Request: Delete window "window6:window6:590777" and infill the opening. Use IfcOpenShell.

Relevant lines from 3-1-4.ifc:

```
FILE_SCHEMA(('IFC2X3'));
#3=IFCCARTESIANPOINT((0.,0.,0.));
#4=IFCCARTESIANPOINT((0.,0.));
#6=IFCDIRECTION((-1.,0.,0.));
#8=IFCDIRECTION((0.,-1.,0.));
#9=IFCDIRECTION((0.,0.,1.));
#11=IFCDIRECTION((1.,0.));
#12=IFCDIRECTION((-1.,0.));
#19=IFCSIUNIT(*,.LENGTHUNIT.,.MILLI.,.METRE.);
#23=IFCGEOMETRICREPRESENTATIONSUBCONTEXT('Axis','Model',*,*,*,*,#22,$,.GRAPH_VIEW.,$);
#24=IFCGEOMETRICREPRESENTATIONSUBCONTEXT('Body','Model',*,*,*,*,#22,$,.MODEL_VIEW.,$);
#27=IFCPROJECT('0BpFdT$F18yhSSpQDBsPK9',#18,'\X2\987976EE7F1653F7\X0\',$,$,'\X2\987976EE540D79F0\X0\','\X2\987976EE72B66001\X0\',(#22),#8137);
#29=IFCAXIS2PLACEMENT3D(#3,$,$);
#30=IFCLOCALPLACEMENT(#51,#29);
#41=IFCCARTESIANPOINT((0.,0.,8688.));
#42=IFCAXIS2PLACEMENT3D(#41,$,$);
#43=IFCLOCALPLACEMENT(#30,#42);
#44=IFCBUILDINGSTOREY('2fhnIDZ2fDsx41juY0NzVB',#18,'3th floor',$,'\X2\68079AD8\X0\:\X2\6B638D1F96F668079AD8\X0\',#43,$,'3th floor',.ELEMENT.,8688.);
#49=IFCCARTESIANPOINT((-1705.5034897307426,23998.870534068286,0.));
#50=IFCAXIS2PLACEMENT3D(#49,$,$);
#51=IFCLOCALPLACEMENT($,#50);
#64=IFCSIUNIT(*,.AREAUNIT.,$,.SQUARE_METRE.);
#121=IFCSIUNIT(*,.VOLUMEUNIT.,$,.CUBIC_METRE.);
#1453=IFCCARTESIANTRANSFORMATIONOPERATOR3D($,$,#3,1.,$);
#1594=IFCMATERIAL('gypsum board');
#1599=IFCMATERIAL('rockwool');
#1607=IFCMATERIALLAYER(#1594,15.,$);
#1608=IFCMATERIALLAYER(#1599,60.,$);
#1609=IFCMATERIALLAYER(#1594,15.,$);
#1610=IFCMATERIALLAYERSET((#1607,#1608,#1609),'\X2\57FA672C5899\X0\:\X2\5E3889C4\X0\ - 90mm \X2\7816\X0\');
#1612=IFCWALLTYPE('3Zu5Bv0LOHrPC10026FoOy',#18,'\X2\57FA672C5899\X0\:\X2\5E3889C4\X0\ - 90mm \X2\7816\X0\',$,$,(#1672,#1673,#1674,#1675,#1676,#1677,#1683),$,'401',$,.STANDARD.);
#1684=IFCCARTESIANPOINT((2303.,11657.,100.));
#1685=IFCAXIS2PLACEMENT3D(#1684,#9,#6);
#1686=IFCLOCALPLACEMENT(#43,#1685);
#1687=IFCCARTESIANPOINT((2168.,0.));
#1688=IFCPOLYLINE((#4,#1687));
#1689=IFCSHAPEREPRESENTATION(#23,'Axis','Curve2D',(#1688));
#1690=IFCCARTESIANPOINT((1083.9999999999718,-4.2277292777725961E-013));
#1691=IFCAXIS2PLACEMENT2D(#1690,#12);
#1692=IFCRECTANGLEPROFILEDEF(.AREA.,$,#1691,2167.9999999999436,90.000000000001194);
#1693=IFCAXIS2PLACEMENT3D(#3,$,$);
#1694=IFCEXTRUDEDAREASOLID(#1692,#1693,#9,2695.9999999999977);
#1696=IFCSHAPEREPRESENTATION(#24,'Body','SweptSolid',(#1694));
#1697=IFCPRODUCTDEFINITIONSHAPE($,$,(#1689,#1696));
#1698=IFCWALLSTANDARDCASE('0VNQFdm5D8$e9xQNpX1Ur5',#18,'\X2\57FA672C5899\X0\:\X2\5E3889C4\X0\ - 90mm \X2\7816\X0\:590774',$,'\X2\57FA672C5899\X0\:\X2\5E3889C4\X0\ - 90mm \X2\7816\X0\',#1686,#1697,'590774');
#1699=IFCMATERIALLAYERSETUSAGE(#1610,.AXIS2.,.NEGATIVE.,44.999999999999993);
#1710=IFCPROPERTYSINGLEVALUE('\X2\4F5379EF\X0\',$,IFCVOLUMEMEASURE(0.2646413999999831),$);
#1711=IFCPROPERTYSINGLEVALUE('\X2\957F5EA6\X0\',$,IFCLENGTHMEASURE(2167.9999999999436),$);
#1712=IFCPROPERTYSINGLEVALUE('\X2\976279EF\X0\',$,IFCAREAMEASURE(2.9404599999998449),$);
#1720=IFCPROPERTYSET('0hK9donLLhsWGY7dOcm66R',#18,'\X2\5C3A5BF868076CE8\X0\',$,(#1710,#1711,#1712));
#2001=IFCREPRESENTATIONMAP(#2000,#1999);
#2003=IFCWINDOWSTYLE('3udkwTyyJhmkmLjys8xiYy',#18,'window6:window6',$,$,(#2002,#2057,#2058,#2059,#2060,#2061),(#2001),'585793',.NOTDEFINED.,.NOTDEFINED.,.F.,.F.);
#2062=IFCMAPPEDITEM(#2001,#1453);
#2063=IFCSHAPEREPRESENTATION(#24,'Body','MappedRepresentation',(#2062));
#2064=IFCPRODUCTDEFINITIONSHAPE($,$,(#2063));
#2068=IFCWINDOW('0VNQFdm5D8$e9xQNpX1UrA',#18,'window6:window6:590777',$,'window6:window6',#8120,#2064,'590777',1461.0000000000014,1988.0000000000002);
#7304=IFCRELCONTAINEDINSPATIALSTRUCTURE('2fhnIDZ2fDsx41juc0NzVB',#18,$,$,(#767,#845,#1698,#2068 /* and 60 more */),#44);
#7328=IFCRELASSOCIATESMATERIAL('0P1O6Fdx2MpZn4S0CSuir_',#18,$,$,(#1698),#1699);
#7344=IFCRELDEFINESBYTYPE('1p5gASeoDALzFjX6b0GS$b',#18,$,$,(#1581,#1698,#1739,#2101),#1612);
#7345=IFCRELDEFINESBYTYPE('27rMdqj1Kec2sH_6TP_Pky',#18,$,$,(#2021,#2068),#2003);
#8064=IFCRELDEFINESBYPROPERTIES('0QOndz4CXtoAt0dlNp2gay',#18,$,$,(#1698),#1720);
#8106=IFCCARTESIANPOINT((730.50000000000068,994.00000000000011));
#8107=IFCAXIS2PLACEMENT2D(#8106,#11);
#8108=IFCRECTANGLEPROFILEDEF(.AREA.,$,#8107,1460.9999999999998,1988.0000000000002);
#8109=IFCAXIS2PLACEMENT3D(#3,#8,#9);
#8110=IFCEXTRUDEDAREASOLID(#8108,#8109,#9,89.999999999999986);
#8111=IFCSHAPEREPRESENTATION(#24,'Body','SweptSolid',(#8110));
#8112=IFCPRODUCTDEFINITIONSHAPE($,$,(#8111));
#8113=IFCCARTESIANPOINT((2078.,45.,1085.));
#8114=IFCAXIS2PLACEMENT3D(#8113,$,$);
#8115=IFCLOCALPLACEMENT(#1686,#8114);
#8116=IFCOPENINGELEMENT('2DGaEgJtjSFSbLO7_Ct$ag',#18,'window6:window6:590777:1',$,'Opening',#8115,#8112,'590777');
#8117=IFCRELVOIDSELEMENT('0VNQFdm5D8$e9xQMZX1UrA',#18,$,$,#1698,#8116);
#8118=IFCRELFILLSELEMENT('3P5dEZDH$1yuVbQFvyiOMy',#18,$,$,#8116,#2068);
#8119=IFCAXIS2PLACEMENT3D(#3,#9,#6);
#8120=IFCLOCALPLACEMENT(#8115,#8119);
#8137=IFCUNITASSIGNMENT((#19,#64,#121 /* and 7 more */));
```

```python
import ifcopenshell
import ifcopenshell.api.feature
import ifcopenshell.api.pset
import ifcopenshell.api.root
import ifcopenshell.geom
import ifcopenshell.util.element
import ifcopenshell.util.shape
import ifcopenshell.util.unit

model = ifcopenshell.open("3-1-4.ifc")
area_scale = ifcopenshell.util.unit.calculate_unit_scale(model, "AREAUNIT")
volume_scale = ifcopenshell.util.unit.calculate_unit_scale(model, "VOLUMEUNIT")
settings = ifcopenshell.geom.settings()


def volume(element):
    """Net volume in cubic metres, openings subtracted."""
    shape = ifcopenshell.geom.create_shape(settings, element)
    return ifcopenshell.util.shape.get_volume(shape.geometry)


window = model.by_id(2068)
opening = window.FillsVoids[0].RelatingOpeningElement
wall = opening.VoidsElements[0].RelatingBuildingElement
before = volume(wall)

ifcopenshell.api.root.remove_product(model, product=window)
ifcopenshell.api.feature.remove_feature(model, feature=opening)

after = volume(wall)
thickness = 0.09  # wall thickness in metres

# Update the wall's stored quantities.
pset = model.by_id(ifcopenshell.util.element.get_pset(wall, "尺寸标注", should_inherit=False)["id"])
ifcopenshell.api.pset.edit_pset(model, pset=pset, properties={
    "体积": model.create_entity("IfcVolumeMeasure", after / volume_scale),
    "面积": model.create_entity("IfcAreaMeasure", after / thickness / area_scale),
})

print(f"wall volume {before:.3f} -> {after:.3f} m3")

model.write("3-1-4-out.ifc")
```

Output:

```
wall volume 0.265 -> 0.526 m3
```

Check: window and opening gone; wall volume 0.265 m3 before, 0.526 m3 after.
